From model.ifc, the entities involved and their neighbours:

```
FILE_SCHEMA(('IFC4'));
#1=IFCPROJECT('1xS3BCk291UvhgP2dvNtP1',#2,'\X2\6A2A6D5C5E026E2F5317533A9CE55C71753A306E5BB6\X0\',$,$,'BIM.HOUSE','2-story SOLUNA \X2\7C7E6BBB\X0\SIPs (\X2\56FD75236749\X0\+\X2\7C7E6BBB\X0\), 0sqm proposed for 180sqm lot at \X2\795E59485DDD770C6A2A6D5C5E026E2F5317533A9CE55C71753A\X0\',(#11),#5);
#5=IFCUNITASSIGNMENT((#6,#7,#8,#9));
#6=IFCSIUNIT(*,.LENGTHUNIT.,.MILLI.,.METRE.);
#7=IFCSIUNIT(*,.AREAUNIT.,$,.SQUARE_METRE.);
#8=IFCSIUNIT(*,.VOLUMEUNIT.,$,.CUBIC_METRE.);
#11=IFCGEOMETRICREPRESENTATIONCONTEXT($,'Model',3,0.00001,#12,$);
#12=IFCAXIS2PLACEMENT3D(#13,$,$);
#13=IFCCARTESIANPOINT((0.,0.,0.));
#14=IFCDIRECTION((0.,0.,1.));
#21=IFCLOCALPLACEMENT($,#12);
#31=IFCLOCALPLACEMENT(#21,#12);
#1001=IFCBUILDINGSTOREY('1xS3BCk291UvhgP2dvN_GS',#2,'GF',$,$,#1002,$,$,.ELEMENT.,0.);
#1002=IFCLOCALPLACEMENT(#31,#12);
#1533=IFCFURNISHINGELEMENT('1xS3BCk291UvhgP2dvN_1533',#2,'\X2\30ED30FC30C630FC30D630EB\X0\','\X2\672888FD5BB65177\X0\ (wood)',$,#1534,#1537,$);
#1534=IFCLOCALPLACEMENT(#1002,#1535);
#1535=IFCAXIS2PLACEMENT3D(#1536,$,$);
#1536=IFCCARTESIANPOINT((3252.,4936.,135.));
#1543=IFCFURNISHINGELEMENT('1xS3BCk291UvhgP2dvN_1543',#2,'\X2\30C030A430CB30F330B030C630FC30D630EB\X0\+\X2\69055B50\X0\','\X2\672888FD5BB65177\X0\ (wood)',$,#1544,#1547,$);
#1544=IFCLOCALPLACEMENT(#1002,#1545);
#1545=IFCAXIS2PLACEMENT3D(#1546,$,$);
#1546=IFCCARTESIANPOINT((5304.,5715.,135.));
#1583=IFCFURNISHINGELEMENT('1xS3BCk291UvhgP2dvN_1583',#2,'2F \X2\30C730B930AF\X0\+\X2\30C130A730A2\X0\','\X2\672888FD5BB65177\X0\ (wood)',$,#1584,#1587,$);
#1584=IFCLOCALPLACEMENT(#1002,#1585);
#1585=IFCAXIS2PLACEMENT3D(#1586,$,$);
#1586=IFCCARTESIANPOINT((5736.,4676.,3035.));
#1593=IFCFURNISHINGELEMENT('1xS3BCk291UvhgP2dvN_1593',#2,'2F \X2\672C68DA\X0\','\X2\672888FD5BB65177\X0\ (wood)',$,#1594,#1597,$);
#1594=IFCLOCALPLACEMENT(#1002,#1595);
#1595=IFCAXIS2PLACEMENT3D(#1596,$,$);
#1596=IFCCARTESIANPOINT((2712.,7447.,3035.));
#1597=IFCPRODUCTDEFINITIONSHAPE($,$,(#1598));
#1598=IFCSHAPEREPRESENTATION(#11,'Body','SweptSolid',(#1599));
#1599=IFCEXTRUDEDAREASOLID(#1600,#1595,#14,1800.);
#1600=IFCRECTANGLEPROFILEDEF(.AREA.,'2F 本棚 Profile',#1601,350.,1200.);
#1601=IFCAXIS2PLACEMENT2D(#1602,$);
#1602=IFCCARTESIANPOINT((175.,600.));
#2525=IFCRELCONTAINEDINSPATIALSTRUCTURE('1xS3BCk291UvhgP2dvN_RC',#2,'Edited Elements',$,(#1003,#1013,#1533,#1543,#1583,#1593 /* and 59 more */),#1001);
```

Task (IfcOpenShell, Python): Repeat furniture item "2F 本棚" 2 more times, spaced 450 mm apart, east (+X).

```python
import numpy as np
import ifcopenshell
import ifcopenshell.api.geometry
import ifcopenshell.api.root
import ifcopenshell.util.element
import ifcopenshell.util.placement

model = ifcopenshell.open("model.ifc")


def reuse_history(source, copy):
    """copy_class also copies each property set's owner history, people and application; keep the originals."""
    for rel in copy.IsDefinedBy:
        if rel.is_a("IfcRelDefinesByProperties") and (history := rel.RelatingPropertyDefinition.OwnerHistory):
            rel.RelatingPropertyDefinition.OwnerHistory = source.OwnerHistory
            ifcopenshell.util.element.remove_deep2(model, history)


source = model.by_guid("1xS3BCk291UvhgP2dvN_1593")
base = ifcopenshell.util.placement.get_local_placement(source.ObjectPlacement)
step = np.array([1.0, 0.0, 0.0]) * 450.0

for i in range(1, 3):
    copy = ifcopenshell.api.root.copy_class(model, product=source)
    copy.Representation = ifcopenshell.util.element.copy_deep(
        model, source.Representation, exclude=["IfcGeometricRepresentationContext", "IfcRepresentationMap"]
    )
    reuse_history(source, copy)
    matrix = base.copy()
    matrix[:3, 3] += i * step
    print("added at", matrix[:3, 3].round(3) + 0.0)
    ifcopenshell.api.geometry.edit_object_placement(model, product=copy, matrix=matrix, is_si=False)

model.write("model_v2.ifc")
```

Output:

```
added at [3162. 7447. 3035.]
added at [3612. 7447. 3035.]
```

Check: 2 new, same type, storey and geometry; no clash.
